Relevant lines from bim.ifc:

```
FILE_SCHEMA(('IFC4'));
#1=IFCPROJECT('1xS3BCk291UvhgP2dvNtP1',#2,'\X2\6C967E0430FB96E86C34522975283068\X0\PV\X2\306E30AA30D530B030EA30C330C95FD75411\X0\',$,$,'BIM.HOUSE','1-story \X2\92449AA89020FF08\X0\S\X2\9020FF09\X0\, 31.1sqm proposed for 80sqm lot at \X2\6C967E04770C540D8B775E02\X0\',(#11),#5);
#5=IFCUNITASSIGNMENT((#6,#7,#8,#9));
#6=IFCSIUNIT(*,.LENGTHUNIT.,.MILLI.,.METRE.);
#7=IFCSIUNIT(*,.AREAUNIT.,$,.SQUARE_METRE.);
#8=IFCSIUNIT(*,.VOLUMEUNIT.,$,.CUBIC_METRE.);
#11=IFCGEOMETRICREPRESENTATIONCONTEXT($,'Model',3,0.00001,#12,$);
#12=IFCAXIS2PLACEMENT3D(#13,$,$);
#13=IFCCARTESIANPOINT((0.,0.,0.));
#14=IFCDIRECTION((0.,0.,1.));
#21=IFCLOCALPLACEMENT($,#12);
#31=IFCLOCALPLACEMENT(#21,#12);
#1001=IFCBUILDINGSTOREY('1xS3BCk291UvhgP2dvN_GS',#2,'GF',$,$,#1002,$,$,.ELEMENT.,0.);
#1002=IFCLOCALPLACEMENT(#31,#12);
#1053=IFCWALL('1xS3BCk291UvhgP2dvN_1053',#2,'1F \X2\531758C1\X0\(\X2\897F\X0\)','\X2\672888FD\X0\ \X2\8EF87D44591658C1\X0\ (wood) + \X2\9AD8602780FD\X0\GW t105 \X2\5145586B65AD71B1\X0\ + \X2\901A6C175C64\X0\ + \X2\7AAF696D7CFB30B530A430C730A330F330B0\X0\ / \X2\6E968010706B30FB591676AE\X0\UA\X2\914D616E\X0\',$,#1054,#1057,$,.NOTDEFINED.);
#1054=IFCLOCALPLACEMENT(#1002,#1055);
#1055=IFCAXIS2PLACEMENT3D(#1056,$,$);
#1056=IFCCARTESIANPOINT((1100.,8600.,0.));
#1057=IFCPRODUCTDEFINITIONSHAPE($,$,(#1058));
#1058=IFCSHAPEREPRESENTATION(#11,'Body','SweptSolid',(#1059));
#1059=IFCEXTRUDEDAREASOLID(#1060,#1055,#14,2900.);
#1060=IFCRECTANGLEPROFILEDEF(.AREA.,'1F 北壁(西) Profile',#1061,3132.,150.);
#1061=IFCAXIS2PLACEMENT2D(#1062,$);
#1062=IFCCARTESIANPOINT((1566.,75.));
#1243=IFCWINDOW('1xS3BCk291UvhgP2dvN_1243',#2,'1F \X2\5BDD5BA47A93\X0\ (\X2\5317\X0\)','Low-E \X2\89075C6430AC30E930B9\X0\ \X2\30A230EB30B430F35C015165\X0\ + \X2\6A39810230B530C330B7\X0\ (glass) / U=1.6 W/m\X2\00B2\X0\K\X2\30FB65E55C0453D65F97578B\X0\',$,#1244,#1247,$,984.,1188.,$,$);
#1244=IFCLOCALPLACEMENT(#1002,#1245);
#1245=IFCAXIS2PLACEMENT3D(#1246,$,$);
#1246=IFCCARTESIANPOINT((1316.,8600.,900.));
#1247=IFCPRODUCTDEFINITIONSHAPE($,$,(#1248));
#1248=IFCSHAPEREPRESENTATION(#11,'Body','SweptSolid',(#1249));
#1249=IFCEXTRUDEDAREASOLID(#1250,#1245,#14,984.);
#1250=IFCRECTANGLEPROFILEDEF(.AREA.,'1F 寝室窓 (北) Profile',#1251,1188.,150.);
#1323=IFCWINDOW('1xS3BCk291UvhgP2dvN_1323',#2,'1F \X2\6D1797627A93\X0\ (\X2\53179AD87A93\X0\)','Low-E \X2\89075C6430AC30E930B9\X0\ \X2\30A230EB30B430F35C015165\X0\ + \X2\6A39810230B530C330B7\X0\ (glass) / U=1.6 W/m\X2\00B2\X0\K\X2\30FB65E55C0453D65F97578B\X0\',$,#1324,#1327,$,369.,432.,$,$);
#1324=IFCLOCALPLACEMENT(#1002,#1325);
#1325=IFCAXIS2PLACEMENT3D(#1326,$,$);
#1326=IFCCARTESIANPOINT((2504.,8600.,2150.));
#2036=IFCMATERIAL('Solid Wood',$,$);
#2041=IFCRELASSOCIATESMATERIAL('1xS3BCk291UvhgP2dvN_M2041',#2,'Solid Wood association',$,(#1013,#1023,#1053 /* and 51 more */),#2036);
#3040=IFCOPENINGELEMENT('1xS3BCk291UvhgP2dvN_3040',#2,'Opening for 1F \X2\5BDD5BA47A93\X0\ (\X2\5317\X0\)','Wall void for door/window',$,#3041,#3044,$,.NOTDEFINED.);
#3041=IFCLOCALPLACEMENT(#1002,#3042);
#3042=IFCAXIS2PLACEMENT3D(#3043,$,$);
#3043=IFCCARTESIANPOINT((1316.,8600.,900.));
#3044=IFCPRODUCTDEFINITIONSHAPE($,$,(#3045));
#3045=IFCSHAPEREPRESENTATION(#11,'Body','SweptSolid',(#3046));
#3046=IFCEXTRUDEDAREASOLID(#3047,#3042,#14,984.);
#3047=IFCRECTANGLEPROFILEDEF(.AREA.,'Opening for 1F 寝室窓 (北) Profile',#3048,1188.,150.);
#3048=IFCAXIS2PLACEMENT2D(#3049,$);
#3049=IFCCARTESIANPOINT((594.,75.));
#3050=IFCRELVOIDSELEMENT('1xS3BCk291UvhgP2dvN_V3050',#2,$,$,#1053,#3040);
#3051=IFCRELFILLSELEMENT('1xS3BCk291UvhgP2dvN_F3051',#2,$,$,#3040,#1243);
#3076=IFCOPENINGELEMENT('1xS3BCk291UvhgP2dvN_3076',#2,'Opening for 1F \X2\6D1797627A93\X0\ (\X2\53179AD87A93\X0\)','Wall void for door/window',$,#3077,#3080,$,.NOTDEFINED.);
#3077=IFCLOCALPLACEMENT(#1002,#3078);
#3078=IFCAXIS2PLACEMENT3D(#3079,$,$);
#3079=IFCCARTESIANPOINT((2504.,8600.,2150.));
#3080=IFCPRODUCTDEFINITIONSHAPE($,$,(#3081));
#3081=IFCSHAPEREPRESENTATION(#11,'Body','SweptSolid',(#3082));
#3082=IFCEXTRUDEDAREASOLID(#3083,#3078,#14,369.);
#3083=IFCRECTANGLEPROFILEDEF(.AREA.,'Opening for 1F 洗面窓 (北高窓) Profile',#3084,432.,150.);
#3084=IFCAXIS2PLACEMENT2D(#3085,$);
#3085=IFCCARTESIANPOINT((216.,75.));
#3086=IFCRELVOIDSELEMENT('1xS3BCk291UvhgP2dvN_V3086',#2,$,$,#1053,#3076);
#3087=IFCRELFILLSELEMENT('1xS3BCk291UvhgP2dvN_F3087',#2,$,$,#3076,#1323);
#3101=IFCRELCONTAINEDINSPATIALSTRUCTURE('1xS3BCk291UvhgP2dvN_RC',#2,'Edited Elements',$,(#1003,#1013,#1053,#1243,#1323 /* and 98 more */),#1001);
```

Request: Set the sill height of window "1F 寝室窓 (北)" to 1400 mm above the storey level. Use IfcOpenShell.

```python
import numpy as np
import ifcopenshell
import ifcopenshell.api.geometry
import ifcopenshell.geom
import ifcopenshell.util.element
import ifcopenshell.util.placement
import ifcopenshell.util.shape
import ifcopenshell.util.unit

model = ifcopenshell.open("bim.ifc")
unit_scale = ifcopenshell.util.unit.calculate_unit_scale(model)

window = model.by_guid("1xS3BCk291UvhgP2dvN_1243")
opening = window.FillsVoids[0].RelatingOpeningElement
storey = ifcopenshell.util.element.get_container(window, ifc_class="IfcBuildingStorey")
level = ifcopenshell.util.placement.get_local_placement(storey.ObjectPlacement)[2, 3]

# The opening's origin need not be at the sill, so measure its lowest point.
shape = ifcopenshell.geom.create_shape(ifcopenshell.geom.settings(), opening)
bottom = ifcopenshell.util.shape.get_shape_bottom_elevation(shape, shape.geometry) / unit_scale
dz = level + 1.4 / unit_scale - bottom

shift = np.array([0.0, 0.0, dz])
# The window is not placed relative to its opening, so move both.
for product in (opening, window):
    matrix = ifcopenshell.util.placement.get_local_placement(product.ObjectPlacement)
    matrix[:3, 3] += shift
    ifcopenshell.api.geometry.edit_object_placement(model, product=product, matrix=matrix, is_si=False)

print(f"moved by {dz * unit_scale:+.3f} m")

model.write("bim_rev.ifc")
```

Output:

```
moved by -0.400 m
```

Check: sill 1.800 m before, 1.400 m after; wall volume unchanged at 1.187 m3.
